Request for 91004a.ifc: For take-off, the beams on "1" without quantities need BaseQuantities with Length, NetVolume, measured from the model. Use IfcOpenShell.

First a look at what the model holds.

```python
import ifcopenshell
import ifcopenshell.util.element
import ifcopenshell.util.unit

model = ifcopenshell.open("91004a.ifc")
print(model.schema)
for unit_type in ("LENGTHUNIT", "AREAUNIT", "VOLUMEUNIT"):
    print(unit_type, ifcopenshell.util.unit.calculate_unit_scale(model, unit_type))
storey = next(s for s in model.by_type("IfcBuildingStorey") if s.Name == "1")
beams = [e for e in ifcopenshell.util.element.get_decomposition(storey) if e.is_a("IfcBeam")]
for e in sorted(beams, key=lambda e: e.id()):
    print(e.id(), e.is_a(), e.Name, list(ifcopenshell.util.element.get_psets(e, qtos_only=True)), sep=" | ")
```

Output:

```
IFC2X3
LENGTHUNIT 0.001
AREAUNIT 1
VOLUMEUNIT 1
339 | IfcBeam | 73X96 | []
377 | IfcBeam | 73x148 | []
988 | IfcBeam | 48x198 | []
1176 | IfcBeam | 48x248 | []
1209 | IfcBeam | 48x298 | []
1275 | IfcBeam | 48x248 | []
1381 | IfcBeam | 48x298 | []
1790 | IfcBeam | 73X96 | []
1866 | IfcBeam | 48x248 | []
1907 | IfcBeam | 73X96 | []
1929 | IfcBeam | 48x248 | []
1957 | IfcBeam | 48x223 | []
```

```python
import ifcopenshell
import ifcopenshell.api.pset
import ifcopenshell.geom
import ifcopenshell.util.element
import ifcopenshell.util.shape
import ifcopenshell.util.unit

model = ifcopenshell.open("91004a.ifc")
unit_scale = ifcopenshell.util.unit.calculate_unit_scale(model)
volume_scale = ifcopenshell.util.unit.calculate_unit_scale(model, "VOLUMEUNIT")
settings = ifcopenshell.geom.settings()

storey = next(s for s in model.by_type("IfcBuildingStorey") if s.Name == "1")
beams = [e for e in ifcopenshell.util.element.get_decomposition(storey) if e.is_a("IfcBeam")]

for e in sorted(beams, key=lambda e: e.id()):
    if ifcopenshell.util.element.get_psets(e, qtos_only=True, should_inherit=False):
        continue
    # Geometry comes back in metres, in the element's own axes.
    shape = ifcopenshell.geom.create_shape(settings, e)
    values = {
        "Length": ifcopenshell.util.shape.get_max_xyz(shape.geometry) / unit_scale,
        "NetVolume": ifcopenshell.util.shape.get_volume(shape.geometry) / volume_scale,
    }
    qto = ifcopenshell.api.pset.add_qto(model, product=e, name="BaseQuantities")
    ifcopenshell.api.pset.edit_qto(model, qto=qto, properties=values)
    print(e.id(), {k: round(v, 3) for k, v in values.items()})

model.write("91004a_rev.ifc")
```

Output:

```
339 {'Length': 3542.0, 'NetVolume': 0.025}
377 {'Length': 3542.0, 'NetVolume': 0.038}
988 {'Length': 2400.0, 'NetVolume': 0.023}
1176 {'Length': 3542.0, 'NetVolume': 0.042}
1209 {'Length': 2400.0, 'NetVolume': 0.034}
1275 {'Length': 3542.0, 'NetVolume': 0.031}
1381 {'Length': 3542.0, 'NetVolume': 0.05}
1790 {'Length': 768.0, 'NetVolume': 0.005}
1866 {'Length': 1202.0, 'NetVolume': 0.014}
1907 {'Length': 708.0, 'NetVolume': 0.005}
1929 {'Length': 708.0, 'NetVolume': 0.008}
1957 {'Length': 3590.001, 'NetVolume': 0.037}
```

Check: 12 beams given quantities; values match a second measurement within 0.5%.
